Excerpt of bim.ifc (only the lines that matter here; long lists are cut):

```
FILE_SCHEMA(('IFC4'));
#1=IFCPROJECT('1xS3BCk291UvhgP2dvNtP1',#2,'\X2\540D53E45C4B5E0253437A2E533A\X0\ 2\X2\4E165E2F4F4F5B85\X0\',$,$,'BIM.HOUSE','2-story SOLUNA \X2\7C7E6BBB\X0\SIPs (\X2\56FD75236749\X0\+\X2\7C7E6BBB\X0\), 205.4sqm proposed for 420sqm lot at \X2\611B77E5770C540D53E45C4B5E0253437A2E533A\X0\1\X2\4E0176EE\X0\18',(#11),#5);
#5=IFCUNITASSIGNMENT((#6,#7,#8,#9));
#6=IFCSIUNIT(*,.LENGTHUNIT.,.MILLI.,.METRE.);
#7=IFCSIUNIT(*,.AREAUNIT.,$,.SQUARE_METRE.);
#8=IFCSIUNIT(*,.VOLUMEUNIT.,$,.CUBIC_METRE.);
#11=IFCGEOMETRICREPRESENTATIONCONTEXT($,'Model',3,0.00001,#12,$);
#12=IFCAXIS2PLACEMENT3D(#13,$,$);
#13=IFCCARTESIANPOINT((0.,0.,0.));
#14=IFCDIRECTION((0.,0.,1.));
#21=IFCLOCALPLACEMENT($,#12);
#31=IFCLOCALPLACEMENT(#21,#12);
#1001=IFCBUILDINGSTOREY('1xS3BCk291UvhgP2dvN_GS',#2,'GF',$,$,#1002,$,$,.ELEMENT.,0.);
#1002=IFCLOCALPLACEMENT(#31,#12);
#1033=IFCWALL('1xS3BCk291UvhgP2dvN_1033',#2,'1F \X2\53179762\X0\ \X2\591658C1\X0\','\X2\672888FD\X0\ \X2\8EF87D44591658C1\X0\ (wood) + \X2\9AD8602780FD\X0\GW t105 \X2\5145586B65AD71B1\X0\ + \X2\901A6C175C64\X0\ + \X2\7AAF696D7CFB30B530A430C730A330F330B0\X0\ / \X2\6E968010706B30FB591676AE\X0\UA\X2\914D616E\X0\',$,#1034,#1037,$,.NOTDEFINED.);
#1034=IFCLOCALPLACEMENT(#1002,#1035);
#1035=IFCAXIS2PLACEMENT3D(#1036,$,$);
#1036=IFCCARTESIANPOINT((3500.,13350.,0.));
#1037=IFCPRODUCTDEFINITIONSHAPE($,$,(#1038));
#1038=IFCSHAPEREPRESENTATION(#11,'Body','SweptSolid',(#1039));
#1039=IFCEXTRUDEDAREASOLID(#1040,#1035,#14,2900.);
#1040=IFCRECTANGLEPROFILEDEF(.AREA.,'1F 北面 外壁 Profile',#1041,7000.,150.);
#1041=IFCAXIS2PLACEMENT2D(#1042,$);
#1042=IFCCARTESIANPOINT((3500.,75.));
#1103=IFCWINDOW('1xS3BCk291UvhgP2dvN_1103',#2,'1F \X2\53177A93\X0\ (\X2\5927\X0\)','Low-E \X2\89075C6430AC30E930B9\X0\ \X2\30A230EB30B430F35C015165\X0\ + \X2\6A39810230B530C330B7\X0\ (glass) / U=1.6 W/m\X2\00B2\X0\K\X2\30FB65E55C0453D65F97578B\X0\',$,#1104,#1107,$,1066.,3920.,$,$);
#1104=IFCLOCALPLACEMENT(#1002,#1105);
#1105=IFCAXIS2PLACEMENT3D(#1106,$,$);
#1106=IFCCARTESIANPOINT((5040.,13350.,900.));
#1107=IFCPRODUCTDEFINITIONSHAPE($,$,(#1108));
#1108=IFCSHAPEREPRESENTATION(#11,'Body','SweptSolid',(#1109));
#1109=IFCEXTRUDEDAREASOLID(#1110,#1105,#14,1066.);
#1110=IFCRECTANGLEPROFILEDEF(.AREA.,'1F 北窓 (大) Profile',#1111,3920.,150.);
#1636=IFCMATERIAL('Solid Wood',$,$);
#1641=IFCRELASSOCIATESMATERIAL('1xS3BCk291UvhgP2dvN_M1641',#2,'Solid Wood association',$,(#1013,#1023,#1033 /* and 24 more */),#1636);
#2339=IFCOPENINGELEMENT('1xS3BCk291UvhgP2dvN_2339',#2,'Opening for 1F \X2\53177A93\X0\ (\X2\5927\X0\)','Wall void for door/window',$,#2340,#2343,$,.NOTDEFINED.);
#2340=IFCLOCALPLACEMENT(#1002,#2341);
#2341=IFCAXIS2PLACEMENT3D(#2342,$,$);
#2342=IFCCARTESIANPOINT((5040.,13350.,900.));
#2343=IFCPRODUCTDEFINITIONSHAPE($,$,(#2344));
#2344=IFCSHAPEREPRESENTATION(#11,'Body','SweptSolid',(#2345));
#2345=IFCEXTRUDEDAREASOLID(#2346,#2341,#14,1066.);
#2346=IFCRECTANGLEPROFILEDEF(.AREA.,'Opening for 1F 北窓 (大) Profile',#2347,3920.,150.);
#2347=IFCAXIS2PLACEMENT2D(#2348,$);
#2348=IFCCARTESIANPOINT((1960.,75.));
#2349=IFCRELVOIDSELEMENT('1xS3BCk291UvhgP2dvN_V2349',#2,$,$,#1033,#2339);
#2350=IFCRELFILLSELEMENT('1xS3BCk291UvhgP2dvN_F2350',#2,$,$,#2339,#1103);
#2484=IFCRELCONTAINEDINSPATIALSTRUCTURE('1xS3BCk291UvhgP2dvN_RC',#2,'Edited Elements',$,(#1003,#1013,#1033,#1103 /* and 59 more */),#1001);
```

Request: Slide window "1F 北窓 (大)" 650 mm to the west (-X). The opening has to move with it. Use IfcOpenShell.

```python
import ifcopenshell
import ifcopenshell.api.geometry
import ifcopenshell.util.placement

model = ifcopenshell.open("bim.ifc")

window = model.by_id(1103)
opening = window.FillsVoids[0].RelatingOpeningElement
wall = opening.VoidsElements[0].RelatingBuildingElement

wall_matrix = ifcopenshell.util.placement.get_local_placement(wall.ObjectPlacement)
shift = wall_matrix[:3, 0] * -650.0
before = ifcopenshell.util.placement.get_local_placement(window.ObjectPlacement)[:3, 3].copy()

# The window is not placed relative to its opening, so move both.
for product in (opening, window):
    matrix = ifcopenshell.util.placement.get_local_placement(product.ObjectPlacement)
    matrix[:3, 3] += shift
    ifcopenshell.api.geometry.edit_object_placement(model, product=product, matrix=matrix, is_si=False)

after = ifcopenshell.util.placement.get_local_placement(window.ObjectPlacement)[:3, 3]
print("window moved by", (after - before).round(3) + 0.0)

model.write("bim-out.ifc")
```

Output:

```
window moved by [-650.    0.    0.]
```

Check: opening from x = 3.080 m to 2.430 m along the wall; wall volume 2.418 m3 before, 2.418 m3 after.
